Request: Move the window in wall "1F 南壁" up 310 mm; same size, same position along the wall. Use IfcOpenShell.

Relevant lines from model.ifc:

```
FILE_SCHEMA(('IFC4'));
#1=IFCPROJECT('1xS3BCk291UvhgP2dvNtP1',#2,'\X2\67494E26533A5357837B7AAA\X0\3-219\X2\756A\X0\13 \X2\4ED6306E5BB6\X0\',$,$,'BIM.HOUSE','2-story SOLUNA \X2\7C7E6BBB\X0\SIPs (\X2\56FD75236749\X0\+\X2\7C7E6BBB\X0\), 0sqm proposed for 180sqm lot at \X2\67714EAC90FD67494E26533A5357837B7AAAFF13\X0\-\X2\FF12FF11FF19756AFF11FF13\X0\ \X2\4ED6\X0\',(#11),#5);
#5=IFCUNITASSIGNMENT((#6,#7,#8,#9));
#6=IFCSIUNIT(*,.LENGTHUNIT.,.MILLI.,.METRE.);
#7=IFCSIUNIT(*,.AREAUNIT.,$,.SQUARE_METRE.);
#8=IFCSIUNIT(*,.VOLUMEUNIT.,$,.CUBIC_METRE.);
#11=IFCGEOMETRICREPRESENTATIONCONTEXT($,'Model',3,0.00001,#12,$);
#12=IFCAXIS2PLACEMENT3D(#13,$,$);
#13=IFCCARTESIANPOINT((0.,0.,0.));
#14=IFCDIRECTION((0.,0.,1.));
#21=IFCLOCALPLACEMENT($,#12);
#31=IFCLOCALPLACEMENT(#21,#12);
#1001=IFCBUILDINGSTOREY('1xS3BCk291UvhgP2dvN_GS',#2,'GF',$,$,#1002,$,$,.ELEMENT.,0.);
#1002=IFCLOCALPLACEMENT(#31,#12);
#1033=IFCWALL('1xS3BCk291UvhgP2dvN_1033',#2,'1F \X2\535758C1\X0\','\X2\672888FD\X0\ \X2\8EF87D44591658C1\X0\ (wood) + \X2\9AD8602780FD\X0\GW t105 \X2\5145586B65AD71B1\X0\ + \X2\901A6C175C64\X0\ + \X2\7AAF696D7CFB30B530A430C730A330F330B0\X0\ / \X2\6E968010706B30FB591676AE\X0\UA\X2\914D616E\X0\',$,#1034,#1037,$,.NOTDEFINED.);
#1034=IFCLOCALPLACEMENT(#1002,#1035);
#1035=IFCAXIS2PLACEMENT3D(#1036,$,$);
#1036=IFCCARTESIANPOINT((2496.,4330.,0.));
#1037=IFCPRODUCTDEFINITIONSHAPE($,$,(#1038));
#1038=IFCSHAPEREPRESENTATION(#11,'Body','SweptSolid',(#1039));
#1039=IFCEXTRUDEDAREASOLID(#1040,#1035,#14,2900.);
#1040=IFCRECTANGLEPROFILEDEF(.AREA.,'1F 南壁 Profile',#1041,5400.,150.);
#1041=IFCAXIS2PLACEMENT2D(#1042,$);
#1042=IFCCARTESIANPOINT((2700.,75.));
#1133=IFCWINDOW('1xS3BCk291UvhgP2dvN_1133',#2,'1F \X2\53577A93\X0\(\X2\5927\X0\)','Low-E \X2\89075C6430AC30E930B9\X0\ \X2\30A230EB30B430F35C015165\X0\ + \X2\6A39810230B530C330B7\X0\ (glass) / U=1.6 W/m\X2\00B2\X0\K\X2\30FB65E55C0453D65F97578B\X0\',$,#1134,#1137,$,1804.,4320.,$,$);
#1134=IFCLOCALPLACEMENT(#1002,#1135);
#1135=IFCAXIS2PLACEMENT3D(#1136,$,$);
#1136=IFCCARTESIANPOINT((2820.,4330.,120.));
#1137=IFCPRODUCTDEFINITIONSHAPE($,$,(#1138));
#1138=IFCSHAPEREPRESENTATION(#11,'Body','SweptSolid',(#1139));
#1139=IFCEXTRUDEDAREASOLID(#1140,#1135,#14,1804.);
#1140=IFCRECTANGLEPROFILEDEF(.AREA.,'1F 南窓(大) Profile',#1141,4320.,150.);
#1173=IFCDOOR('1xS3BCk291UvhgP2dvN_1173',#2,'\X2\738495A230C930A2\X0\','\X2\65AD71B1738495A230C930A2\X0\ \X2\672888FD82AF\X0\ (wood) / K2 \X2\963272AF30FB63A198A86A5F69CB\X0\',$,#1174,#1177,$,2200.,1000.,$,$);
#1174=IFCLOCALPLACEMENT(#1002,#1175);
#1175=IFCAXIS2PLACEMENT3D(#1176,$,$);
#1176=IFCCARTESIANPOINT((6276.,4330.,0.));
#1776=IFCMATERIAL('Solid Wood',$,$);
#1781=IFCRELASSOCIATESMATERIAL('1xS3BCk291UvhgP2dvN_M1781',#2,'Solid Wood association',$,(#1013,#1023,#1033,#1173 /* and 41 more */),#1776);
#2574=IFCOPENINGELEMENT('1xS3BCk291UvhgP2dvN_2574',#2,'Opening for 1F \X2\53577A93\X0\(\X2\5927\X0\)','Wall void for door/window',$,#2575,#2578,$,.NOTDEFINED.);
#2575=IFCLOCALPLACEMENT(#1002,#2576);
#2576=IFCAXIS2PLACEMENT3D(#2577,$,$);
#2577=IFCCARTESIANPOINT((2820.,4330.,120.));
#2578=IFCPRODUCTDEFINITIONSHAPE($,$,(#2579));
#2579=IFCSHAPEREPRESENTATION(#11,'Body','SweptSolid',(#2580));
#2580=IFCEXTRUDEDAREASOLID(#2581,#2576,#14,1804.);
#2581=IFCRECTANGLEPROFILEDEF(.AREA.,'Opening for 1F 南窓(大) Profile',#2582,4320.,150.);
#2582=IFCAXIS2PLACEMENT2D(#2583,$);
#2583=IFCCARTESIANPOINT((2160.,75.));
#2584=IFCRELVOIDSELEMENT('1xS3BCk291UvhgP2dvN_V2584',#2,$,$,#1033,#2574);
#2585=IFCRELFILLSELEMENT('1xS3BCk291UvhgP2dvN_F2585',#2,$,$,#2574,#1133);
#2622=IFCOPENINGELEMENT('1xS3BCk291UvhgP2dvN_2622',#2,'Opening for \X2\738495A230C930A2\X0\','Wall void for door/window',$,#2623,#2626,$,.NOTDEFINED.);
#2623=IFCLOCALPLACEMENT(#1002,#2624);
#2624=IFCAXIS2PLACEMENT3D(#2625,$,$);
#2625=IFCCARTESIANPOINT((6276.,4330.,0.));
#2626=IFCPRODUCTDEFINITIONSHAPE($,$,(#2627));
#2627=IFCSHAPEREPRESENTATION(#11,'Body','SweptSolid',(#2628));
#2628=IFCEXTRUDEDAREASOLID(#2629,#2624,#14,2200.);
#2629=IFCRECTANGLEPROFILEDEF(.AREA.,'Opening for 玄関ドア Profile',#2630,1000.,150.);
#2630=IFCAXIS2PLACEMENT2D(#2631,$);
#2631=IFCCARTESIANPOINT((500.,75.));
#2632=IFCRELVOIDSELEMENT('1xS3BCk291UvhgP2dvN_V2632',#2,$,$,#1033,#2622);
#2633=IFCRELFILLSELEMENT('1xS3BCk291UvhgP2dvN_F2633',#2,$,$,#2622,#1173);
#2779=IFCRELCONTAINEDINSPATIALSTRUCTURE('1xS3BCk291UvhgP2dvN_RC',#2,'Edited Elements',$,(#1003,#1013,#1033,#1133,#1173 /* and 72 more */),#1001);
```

```python
import numpy as np
import ifcopenshell
import ifcopenshell.api.geometry
import ifcopenshell.util.placement
import ifcopenshell.util.unit

model = ifcopenshell.open("model.ifc")
unit_scale = ifcopenshell.util.unit.calculate_unit_scale(model)

window = model.by_guid("1xS3BCk291UvhgP2dvN_1133")
opening = window.FillsVoids[0].RelatingOpeningElement
dz = 0.31 / unit_scale

shift = np.array([0.0, 0.0, dz])
# The window is not placed relative to its opening, so move both.
for product in (opening, window):
    matrix = ifcopenshell.util.placement.get_local_placement(product.ObjectPlacement)
    matrix[:3, 3] += shift
    ifcopenshell.api.geometry.edit_object_placement(model, product=product, matrix=matrix, is_si=False)

print(f"moved by {dz * unit_scale:+.3f} m")

model.write("model_edited.ifc")
```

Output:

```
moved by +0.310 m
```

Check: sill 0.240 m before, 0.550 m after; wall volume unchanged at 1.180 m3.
